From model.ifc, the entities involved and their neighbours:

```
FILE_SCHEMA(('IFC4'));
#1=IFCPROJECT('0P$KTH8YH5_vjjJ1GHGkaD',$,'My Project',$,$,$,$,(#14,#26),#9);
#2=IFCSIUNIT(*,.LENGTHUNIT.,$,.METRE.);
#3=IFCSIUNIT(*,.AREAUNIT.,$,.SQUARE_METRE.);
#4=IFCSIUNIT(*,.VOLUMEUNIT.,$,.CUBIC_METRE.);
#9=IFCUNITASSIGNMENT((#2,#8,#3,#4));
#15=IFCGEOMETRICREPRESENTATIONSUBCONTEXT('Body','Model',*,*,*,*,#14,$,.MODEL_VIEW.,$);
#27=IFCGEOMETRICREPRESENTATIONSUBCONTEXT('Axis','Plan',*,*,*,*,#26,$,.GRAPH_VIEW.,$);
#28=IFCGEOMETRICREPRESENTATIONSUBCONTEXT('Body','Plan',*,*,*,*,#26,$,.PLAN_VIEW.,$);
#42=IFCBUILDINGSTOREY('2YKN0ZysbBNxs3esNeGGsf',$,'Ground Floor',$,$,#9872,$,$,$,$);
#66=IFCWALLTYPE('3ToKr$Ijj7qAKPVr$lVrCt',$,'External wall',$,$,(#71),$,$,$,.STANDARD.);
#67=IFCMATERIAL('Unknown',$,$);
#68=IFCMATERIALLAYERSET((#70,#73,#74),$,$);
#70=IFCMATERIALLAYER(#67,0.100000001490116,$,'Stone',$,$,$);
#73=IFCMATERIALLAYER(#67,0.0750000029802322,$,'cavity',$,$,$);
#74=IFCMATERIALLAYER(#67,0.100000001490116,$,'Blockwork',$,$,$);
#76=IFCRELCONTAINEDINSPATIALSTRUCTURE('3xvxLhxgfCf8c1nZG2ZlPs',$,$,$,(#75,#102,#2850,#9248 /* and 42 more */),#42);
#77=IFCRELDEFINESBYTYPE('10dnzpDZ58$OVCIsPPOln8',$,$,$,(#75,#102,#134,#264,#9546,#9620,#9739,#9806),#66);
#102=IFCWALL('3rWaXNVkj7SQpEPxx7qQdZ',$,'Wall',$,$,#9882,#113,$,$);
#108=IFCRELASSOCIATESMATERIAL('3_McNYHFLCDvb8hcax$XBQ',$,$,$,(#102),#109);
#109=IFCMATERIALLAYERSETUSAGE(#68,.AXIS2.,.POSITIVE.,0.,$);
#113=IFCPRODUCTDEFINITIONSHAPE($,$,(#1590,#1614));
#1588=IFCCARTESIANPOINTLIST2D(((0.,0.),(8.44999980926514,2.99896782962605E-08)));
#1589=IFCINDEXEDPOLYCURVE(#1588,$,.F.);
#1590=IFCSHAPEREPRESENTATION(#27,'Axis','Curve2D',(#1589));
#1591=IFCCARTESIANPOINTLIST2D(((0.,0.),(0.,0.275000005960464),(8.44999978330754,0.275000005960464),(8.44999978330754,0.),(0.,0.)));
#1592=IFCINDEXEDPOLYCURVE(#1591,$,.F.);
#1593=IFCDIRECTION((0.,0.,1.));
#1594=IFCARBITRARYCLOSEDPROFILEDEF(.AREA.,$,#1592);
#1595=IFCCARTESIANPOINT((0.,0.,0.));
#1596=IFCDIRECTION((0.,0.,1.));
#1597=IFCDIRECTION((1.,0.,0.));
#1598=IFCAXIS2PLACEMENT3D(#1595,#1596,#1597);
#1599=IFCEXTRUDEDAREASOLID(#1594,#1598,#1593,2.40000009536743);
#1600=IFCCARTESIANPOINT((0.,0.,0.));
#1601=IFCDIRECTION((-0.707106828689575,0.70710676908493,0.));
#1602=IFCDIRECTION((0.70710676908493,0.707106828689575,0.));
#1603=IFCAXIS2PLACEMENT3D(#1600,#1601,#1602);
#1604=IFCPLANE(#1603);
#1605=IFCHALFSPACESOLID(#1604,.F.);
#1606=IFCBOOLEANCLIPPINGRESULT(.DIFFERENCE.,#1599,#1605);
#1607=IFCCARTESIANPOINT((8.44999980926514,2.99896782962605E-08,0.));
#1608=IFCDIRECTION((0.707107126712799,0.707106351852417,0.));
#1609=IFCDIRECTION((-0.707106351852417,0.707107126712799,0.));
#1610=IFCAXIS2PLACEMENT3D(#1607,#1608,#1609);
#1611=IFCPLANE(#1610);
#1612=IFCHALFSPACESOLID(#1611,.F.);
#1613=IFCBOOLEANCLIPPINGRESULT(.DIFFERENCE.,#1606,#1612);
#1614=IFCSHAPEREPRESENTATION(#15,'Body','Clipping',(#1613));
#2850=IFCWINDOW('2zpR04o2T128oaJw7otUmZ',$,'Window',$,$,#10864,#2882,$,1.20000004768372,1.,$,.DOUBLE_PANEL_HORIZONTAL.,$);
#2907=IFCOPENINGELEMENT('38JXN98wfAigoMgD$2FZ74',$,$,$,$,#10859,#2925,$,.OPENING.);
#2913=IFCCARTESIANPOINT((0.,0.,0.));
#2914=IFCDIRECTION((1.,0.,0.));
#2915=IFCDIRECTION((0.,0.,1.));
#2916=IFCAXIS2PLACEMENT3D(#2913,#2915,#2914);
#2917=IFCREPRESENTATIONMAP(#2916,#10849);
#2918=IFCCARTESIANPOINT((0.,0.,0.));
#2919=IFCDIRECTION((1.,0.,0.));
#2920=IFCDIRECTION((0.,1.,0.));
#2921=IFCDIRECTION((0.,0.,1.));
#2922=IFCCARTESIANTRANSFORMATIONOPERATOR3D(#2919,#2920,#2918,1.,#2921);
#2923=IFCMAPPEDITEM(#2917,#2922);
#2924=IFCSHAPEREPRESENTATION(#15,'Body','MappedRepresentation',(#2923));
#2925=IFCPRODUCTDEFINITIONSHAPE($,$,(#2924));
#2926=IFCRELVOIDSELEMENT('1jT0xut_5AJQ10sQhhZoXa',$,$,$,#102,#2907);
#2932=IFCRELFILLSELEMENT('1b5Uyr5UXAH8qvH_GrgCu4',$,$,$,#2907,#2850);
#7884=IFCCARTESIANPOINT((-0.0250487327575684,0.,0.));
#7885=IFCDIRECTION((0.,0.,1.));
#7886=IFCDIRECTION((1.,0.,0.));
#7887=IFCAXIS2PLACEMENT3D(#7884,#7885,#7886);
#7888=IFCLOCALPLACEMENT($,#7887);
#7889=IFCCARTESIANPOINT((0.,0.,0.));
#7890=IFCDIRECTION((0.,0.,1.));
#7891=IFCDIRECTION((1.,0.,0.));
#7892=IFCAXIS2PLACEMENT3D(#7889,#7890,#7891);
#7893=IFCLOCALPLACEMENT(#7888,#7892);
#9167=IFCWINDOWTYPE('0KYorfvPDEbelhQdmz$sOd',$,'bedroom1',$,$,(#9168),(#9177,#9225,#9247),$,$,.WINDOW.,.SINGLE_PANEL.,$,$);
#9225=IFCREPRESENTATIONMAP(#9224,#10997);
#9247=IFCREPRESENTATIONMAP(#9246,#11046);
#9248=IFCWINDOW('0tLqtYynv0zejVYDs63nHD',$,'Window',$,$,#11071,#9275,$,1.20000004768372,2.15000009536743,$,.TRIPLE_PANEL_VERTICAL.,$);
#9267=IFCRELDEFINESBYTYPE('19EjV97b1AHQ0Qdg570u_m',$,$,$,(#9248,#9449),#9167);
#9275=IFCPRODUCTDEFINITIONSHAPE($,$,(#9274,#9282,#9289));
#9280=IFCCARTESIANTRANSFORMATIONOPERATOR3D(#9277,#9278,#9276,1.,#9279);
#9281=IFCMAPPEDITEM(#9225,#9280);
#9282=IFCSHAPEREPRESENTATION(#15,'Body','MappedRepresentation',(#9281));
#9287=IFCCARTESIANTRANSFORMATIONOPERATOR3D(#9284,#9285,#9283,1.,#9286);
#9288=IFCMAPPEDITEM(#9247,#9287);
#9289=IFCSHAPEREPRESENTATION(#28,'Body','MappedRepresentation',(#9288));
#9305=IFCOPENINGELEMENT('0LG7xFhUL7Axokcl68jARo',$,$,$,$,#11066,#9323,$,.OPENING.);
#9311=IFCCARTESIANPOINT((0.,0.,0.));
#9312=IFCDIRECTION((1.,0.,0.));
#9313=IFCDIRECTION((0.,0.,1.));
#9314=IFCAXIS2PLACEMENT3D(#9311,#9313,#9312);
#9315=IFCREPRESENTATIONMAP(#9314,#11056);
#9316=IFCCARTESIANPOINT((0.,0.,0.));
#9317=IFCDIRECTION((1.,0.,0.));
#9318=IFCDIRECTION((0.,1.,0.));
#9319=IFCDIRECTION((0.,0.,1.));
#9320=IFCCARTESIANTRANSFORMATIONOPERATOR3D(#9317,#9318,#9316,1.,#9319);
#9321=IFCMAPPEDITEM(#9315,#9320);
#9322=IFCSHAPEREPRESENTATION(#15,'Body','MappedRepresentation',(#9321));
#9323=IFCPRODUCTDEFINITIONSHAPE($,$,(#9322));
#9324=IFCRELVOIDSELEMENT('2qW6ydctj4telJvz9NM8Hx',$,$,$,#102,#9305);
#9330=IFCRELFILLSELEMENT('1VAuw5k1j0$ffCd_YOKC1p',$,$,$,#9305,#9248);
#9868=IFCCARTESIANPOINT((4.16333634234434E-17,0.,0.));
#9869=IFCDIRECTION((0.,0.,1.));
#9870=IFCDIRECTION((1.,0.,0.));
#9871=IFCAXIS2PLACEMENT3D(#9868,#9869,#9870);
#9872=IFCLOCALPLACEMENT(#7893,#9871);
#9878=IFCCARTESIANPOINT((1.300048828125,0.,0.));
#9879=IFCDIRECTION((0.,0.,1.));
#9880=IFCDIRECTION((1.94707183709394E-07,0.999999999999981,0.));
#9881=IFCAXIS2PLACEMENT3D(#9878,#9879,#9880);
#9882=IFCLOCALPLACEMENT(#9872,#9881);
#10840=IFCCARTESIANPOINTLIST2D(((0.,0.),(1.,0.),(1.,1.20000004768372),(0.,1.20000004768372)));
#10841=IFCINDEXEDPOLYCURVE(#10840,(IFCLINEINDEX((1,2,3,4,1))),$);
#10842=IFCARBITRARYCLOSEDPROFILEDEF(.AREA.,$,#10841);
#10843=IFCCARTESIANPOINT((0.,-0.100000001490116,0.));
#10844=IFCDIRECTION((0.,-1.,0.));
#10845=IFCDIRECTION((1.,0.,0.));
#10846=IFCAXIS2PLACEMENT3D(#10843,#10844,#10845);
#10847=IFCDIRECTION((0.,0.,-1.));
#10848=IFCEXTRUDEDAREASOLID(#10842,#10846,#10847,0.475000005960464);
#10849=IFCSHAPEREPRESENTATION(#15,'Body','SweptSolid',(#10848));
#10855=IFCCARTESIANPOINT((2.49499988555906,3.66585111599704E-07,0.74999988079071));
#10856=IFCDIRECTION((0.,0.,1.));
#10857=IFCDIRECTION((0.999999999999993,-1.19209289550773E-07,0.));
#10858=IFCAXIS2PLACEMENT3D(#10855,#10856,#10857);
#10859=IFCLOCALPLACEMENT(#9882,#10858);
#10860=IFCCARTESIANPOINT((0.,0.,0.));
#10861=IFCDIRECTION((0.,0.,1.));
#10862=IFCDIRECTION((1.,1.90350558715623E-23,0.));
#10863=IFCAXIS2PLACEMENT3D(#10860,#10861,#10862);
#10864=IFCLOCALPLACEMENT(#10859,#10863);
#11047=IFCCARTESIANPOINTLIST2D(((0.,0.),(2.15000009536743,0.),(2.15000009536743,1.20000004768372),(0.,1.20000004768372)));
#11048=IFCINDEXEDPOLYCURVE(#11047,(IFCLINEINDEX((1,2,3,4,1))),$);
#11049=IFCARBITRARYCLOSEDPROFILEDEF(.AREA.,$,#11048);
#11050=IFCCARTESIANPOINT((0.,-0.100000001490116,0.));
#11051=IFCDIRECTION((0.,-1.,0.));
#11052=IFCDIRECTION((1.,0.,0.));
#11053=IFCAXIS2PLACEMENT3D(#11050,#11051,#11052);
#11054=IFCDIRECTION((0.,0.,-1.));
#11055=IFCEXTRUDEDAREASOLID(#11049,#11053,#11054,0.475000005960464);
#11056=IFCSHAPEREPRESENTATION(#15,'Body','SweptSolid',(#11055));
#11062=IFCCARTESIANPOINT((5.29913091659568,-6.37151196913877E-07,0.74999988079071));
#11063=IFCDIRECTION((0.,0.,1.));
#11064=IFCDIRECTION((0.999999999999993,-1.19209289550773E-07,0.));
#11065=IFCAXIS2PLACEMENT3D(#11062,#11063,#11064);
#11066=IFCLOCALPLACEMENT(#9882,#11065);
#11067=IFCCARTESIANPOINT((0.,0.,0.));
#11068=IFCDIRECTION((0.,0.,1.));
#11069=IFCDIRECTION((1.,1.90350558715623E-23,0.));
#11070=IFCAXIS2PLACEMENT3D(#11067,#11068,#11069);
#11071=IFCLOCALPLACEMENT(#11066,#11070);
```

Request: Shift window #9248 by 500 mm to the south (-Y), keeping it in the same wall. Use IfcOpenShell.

```python
import ifcopenshell
import ifcopenshell.api.geometry
import ifcopenshell.util.placement

model = ifcopenshell.open("model.ifc")

window = model.by_guid("0tLqtYynv0zejVYDs63nHD")
opening = window.FillsVoids[0].RelatingOpeningElement
wall = opening.VoidsElements[0].RelatingBuildingElement

wall_matrix = ifcopenshell.util.placement.get_local_placement(wall.ObjectPlacement)
shift = wall_matrix[:3, 0] * -0.5
before = ifcopenshell.util.placement.get_local_placement(window.ObjectPlacement)[:3, 3].copy()

# The window is placed relative to its opening, so it follows when the opening moves.
matrix = ifcopenshell.util.placement.get_local_placement(opening.ObjectPlacement)
matrix[:3, 3] += shift
ifcopenshell.api.geometry.edit_object_placement(
    model, product=opening, matrix=matrix, is_si=False, should_transform_children=True
)

after = ifcopenshell.util.placement.get_local_placement(window.ObjectPlacement)[:3, 3]
print("window moved by", (after - before).round(3) + 0.0)

model.write("model_rev.ifc")
```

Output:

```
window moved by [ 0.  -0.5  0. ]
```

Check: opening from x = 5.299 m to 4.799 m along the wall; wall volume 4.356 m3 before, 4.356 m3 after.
